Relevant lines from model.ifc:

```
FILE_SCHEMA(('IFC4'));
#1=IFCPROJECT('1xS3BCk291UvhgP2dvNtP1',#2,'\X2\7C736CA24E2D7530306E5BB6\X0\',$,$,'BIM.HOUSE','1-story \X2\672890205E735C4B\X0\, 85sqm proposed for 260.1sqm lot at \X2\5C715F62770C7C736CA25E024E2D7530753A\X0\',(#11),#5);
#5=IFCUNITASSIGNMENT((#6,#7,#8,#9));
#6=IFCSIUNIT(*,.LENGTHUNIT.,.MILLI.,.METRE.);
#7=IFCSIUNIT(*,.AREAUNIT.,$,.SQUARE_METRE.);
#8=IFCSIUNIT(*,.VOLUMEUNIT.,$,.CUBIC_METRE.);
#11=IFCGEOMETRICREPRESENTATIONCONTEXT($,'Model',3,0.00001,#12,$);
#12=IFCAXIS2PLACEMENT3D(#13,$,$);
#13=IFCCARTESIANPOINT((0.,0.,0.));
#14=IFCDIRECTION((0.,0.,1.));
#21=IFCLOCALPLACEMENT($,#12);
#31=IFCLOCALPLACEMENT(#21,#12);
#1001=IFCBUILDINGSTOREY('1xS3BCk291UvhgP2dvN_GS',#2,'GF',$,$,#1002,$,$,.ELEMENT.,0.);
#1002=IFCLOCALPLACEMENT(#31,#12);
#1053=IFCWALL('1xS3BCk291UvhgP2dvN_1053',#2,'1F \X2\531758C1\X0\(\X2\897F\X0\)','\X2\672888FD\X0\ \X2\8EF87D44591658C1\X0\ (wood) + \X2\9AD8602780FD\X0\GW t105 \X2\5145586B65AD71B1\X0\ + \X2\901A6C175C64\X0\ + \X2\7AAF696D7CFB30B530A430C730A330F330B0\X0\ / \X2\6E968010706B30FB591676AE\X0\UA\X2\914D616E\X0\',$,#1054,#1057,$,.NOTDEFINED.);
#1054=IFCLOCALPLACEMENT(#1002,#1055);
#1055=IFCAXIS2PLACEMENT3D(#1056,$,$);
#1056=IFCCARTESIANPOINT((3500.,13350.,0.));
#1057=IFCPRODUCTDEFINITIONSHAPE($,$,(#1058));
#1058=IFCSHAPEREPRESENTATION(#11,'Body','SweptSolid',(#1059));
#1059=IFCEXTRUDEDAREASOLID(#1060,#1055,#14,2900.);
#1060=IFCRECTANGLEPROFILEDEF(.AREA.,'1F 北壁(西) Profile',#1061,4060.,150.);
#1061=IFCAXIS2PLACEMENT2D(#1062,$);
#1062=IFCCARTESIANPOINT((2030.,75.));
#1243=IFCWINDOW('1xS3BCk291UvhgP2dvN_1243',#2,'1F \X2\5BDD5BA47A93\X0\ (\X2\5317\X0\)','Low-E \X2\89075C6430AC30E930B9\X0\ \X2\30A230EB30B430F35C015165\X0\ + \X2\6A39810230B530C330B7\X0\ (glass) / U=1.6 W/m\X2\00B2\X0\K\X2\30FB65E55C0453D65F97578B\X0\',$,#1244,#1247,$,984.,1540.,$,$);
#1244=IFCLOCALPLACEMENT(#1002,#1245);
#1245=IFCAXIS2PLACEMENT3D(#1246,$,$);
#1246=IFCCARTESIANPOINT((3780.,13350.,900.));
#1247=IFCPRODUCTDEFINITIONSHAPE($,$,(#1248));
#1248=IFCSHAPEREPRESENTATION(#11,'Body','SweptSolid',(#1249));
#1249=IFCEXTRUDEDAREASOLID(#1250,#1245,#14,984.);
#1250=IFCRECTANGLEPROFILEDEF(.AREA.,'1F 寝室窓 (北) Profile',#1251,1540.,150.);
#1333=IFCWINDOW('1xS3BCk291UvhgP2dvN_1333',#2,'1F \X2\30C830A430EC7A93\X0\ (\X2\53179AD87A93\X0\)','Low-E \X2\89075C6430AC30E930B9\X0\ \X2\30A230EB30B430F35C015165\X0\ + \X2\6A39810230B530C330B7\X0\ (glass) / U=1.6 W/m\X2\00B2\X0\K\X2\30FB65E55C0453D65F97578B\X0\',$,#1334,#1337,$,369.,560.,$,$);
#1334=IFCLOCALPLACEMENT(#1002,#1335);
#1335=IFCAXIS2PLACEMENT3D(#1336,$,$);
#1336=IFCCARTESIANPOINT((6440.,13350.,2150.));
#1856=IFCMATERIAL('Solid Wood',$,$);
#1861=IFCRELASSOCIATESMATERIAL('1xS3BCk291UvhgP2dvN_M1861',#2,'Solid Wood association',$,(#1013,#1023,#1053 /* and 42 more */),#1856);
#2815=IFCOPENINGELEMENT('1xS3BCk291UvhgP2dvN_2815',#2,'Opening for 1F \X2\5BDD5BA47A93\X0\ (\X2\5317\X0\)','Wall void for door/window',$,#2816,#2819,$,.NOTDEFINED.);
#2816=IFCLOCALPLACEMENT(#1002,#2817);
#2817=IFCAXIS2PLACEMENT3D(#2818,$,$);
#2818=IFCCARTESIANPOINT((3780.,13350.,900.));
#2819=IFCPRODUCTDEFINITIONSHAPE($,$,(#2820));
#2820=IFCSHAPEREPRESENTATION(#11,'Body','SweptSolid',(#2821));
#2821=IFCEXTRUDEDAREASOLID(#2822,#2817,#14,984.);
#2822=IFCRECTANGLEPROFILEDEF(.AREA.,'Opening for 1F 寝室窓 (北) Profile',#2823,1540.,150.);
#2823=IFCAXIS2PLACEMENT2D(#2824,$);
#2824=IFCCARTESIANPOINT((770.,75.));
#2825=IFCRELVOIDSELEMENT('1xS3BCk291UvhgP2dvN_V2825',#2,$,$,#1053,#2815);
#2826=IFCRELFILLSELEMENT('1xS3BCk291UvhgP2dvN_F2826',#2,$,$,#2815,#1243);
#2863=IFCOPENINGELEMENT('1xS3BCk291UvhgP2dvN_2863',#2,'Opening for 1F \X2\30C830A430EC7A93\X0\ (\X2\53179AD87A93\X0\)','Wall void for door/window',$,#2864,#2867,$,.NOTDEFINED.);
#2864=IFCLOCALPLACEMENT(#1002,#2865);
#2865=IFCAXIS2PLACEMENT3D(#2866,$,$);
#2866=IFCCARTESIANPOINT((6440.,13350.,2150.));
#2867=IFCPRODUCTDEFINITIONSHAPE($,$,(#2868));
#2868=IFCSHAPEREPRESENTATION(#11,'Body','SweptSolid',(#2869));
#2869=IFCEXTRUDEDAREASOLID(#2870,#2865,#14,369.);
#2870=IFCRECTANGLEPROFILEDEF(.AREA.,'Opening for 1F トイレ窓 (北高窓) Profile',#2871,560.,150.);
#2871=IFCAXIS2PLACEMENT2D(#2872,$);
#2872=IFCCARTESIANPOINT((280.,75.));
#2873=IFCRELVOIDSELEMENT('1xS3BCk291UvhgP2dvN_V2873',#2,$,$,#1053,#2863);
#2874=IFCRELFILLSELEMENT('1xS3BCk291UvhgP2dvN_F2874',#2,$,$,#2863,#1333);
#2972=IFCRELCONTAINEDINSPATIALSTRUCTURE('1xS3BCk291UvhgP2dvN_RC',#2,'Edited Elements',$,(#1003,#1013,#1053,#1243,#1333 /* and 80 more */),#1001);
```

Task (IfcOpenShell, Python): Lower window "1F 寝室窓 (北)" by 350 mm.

```python
import numpy as np
import ifcopenshell
import ifcopenshell.api.geometry
import ifcopenshell.util.placement
import ifcopenshell.util.unit

model = ifcopenshell.open("model.ifc")
unit_scale = ifcopenshell.util.unit.calculate_unit_scale(model)

window = model.by_guid("1xS3BCk291UvhgP2dvN_1243")
opening = window.FillsVoids[0].RelatingOpeningElement
dz = -0.35 / unit_scale

shift = np.array([0.0, 0.0, dz])
# The window is not placed relative to its opening, so move both.
for product in (opening, window):
    matrix = ifcopenshell.util.placement.get_local_placement(product.ObjectPlacement)
    matrix[:3, 3] += shift
    ifcopenshell.api.geometry.edit_object_placement(model, product=product, matrix=matrix, is_si=False)

print(f"moved by {dz * unit_scale:+.3f} m")

model.write("model-out.ifc")
```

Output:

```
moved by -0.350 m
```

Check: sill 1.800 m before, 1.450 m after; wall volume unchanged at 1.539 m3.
